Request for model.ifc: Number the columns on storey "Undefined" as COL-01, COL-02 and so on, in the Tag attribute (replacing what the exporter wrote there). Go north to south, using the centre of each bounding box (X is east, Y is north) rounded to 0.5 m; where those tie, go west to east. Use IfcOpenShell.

First a look at what the model holds.

```python
import ifcopenshell
import ifcopenshell.util.element
import ifcopenshell.util.placement

model = ifcopenshell.open("model.ifc")
print(model.schema)
storey = next(s for s in model.by_type("IfcBuildingStorey") if s.Name == "Undefined")
columns = [e for e in ifcopenshell.util.element.get_decomposition(storey) if e.is_a("IfcColumn")]
for e in sorted(columns, key=lambda e: e.id()):
    origin = ifcopenshell.util.placement.get_local_placement(e.ObjectPlacement)[:3, 3]
    print(e.id(), e.Tag, e.Name, origin.round(2) + 0.0, sep=" | ")
```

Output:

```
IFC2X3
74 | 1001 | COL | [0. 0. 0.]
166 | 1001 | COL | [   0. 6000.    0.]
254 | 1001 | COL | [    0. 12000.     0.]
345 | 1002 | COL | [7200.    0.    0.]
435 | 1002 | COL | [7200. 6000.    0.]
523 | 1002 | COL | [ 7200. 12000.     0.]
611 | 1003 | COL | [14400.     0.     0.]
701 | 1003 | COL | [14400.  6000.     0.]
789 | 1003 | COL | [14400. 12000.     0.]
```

```python
import ifcopenshell
import ifcopenshell.geom
import ifcopenshell.util.element
import ifcopenshell.util.shape

model = ifcopenshell.open("model.ifc")
settings = ifcopenshell.geom.settings()
settings.set("use-world-coords", True)


def centre(element):
    shape = ifcopenshell.geom.create_shape(settings, element)
    return ifcopenshell.util.shape.get_bbox_centroid(shape.geometry)


storey = next(s for s in model.by_type("IfcBuildingStorey") if s.Name == "Undefined")
columns = [e for e in ifcopenshell.util.element.get_decomposition(storey) if e.is_a("IfcColumn")]

# Insertion points can sit at a corner or the storey origin, so sort by the geometry (in metres).
centres = {e: centre(e) for e in columns}
columns.sort(key=lambda e: (-round(centres[e][1] / 0.5), centres[e][0]))

for i, e in enumerate(columns, start=1):
    number = f"COL-{i:02d}"
    e.Tag = number
    print(e.id(), number)

model.write("model-out.ifc")
```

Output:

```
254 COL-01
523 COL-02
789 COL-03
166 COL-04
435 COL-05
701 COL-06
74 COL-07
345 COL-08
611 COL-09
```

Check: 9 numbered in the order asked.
